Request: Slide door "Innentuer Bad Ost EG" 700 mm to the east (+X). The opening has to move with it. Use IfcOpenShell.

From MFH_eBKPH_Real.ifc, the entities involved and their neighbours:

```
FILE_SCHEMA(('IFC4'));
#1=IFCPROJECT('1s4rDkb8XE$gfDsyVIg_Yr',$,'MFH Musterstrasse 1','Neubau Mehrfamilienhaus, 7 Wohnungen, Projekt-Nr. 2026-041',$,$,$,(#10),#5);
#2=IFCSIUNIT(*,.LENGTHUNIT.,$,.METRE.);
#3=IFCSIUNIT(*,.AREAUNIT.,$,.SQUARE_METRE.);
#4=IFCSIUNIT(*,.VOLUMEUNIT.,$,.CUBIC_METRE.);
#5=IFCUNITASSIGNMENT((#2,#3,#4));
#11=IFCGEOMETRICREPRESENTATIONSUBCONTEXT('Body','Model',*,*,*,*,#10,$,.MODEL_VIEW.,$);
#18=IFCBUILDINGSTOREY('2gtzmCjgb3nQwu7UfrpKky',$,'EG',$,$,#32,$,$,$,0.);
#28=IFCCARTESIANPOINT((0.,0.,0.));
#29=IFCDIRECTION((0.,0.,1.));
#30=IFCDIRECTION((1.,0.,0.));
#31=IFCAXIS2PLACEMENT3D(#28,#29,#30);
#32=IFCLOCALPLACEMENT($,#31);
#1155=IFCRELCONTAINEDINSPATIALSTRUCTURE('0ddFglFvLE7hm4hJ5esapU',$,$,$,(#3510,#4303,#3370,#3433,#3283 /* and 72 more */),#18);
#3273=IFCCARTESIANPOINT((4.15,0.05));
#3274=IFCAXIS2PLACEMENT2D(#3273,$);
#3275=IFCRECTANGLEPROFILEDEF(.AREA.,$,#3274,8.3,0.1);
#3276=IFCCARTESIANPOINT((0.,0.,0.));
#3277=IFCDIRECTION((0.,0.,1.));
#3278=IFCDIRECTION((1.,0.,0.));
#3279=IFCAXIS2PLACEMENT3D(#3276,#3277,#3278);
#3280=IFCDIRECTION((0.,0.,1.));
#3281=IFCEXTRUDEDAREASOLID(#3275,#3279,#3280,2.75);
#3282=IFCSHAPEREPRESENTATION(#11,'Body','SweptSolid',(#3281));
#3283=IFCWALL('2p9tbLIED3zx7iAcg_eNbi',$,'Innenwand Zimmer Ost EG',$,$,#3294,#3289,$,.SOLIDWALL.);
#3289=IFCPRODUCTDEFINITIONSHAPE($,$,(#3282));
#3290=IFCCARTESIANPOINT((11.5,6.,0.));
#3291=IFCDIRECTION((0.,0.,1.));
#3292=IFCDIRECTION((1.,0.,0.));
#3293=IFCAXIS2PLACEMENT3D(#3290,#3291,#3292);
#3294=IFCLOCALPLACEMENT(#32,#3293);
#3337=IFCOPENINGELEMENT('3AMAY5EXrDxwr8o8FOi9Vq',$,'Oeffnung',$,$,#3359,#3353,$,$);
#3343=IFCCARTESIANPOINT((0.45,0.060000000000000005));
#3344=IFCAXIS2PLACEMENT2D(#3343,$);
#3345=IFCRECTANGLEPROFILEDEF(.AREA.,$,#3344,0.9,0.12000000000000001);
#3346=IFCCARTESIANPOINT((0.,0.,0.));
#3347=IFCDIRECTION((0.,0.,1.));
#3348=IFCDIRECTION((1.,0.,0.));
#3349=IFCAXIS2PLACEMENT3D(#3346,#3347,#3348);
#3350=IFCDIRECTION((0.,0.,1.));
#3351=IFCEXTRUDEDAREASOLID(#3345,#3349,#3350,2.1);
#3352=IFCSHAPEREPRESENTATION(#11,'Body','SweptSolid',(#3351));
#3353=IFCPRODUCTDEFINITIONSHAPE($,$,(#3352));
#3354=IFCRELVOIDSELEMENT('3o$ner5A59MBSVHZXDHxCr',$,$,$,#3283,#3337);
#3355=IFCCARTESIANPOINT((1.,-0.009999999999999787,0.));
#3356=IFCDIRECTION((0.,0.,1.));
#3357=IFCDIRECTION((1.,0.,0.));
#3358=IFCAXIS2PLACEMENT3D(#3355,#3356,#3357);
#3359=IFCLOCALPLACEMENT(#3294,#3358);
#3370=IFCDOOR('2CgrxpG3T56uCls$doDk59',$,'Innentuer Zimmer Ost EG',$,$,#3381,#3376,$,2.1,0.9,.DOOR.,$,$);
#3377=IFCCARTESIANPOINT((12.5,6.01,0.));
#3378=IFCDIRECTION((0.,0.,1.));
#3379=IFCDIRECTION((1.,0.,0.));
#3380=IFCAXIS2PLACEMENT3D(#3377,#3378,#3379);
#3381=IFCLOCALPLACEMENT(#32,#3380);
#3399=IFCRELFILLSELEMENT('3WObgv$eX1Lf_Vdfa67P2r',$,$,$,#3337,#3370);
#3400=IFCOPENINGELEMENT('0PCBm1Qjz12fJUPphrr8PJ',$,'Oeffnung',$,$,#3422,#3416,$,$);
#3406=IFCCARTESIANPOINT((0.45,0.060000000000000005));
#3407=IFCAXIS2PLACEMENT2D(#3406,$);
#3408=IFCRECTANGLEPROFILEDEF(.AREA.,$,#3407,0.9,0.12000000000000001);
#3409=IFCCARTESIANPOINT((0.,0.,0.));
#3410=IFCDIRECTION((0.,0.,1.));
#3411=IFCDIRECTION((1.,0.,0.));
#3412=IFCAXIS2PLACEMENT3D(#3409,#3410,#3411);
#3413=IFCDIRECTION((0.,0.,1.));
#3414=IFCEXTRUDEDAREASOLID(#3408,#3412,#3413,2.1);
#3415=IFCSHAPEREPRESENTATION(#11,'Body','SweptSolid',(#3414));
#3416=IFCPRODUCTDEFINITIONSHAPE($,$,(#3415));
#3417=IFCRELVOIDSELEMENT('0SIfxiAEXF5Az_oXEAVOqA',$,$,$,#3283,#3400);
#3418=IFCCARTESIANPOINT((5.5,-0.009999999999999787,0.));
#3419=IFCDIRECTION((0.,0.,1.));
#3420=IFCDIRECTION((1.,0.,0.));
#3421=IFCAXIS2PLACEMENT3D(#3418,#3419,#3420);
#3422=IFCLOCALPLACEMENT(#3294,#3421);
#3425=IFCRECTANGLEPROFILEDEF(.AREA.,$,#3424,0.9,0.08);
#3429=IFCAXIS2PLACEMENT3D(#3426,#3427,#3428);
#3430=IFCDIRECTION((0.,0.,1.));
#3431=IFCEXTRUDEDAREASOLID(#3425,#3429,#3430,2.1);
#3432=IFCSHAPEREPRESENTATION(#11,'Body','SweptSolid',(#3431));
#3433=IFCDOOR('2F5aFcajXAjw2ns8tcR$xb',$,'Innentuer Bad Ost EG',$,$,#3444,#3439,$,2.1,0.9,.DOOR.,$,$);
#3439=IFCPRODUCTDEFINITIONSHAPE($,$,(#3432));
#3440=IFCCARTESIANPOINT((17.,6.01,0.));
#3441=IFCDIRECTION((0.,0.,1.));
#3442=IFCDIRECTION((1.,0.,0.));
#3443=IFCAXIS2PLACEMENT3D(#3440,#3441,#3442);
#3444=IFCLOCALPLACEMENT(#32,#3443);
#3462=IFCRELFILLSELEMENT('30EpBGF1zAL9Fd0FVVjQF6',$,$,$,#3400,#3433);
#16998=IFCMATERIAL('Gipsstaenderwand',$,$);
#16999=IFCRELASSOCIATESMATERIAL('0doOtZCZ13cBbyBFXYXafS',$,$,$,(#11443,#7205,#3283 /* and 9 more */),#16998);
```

```python
import ifcopenshell
import ifcopenshell.api.geometry
import ifcopenshell.util.placement
import ifcopenshell.util.unit

model = ifcopenshell.open("MFH_eBKPH_Real.ifc")
unit_scale = ifcopenshell.util.unit.calculate_unit_scale(model)

door = model.by_guid("2F5aFcajXAjw2ns8tcR$xb")
opening = door.FillsVoids[0].RelatingOpeningElement
wall = opening.VoidsElements[0].RelatingBuildingElement

wall_matrix = ifcopenshell.util.placement.get_local_placement(wall.ObjectPlacement)
shift = wall_matrix[:3, 0] * 0.7 / unit_scale
before = ifcopenshell.util.placement.get_local_placement(door.ObjectPlacement)[:3, 3].copy()

# The door is not placed relative to its opening, so move both.
for product in (opening, door):
    matrix = ifcopenshell.util.placement.get_local_placement(product.ObjectPlacement)
    matrix[:3, 3] += shift
    ifcopenshell.api.geometry.edit_object_placement(model, product=product, matrix=matrix, is_si=False)

after = ifcopenshell.util.placement.get_local_placement(door.ObjectPlacement)[:3, 3]
print("door moved by", (after - before).round(3) + 0.0)

model.write("MFH_eBKPH_Real_updated.ifc")
```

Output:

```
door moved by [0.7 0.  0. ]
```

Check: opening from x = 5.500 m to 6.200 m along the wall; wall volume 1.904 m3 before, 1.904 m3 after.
